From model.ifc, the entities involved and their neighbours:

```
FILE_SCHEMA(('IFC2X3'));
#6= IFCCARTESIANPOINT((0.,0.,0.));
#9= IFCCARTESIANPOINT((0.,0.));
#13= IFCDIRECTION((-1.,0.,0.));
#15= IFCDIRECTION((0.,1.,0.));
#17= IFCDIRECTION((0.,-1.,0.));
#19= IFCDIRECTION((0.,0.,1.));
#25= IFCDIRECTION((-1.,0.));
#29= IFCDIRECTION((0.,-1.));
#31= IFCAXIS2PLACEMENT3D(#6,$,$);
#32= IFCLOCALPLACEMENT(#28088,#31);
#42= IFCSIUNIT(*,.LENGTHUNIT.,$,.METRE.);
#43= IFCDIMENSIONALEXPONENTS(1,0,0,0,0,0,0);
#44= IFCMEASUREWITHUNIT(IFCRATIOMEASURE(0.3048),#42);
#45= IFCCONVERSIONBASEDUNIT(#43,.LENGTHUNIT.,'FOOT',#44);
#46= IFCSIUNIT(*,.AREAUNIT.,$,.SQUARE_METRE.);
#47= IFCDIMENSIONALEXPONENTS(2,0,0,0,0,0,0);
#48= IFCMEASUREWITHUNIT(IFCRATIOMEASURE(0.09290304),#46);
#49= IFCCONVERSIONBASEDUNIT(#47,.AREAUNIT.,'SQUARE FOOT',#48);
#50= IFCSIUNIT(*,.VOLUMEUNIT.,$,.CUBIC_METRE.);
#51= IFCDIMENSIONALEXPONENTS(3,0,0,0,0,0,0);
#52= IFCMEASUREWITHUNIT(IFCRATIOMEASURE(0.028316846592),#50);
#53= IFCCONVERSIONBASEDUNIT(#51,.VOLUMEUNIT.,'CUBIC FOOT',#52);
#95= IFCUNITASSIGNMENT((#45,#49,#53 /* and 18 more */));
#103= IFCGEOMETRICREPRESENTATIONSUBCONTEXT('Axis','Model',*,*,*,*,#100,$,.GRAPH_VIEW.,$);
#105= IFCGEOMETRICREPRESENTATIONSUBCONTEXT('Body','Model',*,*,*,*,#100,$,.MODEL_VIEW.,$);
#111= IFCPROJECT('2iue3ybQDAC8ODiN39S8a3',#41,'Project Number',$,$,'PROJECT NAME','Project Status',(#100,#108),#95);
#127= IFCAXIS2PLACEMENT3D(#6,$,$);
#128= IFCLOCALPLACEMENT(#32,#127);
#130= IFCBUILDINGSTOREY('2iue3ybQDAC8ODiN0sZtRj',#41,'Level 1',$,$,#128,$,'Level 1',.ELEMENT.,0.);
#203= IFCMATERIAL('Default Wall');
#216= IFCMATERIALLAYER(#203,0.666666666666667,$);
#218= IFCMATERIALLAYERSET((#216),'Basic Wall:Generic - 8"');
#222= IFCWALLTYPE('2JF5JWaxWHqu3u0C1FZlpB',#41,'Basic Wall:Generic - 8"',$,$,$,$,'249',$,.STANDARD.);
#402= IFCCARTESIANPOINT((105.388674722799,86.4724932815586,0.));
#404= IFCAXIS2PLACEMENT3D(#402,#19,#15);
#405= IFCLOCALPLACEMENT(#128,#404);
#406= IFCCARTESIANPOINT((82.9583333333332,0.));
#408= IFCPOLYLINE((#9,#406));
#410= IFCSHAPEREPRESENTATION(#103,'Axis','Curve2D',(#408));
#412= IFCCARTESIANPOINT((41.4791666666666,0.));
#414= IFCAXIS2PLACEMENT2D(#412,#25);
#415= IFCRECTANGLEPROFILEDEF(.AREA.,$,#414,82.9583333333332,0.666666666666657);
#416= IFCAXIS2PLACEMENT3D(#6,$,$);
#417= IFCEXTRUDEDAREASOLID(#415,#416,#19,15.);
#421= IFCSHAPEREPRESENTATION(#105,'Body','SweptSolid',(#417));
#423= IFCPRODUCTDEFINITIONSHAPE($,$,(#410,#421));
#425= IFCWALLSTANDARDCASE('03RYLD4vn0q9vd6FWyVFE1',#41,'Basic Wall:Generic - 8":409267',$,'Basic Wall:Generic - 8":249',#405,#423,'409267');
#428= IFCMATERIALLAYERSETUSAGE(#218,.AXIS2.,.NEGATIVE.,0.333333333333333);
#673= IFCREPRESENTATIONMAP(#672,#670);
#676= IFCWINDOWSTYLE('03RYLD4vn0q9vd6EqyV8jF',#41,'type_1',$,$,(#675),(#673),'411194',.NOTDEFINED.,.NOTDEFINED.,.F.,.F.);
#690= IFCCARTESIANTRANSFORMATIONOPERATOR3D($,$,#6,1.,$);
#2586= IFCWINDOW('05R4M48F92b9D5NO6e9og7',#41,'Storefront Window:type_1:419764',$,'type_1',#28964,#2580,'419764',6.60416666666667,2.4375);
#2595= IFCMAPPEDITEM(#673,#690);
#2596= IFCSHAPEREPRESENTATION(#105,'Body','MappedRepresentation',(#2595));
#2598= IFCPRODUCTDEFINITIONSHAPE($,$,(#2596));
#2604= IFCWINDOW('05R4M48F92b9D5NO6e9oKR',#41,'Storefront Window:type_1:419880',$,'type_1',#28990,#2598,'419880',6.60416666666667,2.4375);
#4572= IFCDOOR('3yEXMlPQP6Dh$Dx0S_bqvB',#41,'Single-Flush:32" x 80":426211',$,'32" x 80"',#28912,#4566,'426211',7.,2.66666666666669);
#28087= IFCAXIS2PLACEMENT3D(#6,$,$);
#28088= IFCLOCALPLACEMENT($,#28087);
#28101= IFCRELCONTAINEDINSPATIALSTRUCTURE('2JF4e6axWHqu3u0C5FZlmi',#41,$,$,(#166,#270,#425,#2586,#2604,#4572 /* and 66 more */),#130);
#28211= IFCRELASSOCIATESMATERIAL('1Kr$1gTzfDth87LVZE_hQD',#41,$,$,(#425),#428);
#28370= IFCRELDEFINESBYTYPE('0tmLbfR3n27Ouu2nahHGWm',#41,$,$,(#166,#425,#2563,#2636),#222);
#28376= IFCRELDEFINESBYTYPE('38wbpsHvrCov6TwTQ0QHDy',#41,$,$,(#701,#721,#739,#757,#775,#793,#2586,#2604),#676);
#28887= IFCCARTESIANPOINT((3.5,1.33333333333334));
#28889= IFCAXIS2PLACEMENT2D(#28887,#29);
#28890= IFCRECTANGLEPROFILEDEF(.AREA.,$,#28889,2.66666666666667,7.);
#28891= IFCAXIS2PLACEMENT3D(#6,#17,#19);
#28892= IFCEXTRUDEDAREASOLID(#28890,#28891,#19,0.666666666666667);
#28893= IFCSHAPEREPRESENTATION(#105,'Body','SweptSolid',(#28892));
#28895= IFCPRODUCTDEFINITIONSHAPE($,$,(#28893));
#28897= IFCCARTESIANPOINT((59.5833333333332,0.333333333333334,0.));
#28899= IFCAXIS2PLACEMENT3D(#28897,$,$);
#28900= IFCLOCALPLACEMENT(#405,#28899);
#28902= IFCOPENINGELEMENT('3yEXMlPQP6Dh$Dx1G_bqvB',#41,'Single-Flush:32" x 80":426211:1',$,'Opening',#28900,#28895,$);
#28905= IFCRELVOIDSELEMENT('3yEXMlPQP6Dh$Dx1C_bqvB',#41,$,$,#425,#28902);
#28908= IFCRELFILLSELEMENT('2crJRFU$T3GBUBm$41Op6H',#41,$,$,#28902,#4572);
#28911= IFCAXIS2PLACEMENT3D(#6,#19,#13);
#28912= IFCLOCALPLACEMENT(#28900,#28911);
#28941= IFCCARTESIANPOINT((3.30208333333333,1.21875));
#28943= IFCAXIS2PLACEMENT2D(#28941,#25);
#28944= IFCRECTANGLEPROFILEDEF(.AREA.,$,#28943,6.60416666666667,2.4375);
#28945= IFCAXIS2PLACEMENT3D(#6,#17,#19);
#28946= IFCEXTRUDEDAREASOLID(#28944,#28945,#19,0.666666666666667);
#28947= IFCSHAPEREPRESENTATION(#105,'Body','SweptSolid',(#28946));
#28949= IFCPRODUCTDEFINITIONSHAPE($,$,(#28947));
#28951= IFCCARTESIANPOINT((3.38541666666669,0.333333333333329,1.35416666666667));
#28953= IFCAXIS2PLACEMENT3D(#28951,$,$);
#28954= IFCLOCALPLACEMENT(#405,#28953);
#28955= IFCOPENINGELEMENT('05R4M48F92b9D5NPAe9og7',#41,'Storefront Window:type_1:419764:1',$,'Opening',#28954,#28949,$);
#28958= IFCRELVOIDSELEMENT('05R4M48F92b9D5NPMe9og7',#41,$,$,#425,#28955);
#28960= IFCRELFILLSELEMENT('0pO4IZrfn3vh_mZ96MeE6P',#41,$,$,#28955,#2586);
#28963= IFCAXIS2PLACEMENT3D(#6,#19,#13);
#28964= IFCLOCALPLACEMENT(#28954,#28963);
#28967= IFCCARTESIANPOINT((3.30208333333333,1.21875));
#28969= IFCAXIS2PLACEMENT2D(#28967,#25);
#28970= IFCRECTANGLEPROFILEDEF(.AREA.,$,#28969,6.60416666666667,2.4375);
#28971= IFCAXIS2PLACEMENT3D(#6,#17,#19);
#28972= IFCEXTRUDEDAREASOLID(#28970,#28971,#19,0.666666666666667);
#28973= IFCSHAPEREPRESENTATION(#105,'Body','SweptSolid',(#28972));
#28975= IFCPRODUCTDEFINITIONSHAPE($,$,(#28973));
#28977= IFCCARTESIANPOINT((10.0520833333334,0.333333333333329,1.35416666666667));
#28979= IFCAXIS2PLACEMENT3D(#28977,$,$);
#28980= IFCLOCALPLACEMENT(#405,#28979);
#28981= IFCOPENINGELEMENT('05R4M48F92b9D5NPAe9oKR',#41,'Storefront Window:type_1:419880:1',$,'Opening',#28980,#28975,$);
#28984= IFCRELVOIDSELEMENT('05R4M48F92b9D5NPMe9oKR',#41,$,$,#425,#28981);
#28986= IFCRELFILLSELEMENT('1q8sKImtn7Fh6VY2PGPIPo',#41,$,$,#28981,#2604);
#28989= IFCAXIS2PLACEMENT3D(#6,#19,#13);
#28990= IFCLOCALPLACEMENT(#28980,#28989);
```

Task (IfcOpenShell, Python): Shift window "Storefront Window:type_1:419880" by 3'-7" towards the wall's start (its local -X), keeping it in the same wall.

```python
import ifcopenshell
import ifcopenshell.api.geometry
import ifcopenshell.util.placement
import ifcopenshell.util.unit

model = ifcopenshell.open("model.ifc")
unit_scale = ifcopenshell.util.unit.calculate_unit_scale(model)

window = model.by_id(2604)
opening = window.FillsVoids[0].RelatingOpeningElement
wall = opening.VoidsElements[0].RelatingBuildingElement

wall_matrix = ifcopenshell.util.placement.get_local_placement(wall.ObjectPlacement)
shift = wall_matrix[:3, 0] * -43 * 0.0254 / unit_scale
before = ifcopenshell.util.placement.get_local_placement(window.ObjectPlacement)[:3, 3].copy()

# The window is placed relative to its opening, so it follows when the opening moves.
matrix = ifcopenshell.util.placement.get_local_placement(opening.ObjectPlacement)
matrix[:3, 3] += shift
ifcopenshell.api.geometry.edit_object_placement(
    model, product=opening, matrix=matrix, is_si=False, should_transform_children=True
)

after = ifcopenshell.util.placement.get_local_placement(window.ObjectPlacement)[:3, 3]
print("window moved by", (after - before).round(3) + 0.0)

model.write("model_v2.ifc")
```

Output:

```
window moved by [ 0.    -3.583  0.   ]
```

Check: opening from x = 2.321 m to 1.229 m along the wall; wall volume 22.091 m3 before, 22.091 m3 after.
